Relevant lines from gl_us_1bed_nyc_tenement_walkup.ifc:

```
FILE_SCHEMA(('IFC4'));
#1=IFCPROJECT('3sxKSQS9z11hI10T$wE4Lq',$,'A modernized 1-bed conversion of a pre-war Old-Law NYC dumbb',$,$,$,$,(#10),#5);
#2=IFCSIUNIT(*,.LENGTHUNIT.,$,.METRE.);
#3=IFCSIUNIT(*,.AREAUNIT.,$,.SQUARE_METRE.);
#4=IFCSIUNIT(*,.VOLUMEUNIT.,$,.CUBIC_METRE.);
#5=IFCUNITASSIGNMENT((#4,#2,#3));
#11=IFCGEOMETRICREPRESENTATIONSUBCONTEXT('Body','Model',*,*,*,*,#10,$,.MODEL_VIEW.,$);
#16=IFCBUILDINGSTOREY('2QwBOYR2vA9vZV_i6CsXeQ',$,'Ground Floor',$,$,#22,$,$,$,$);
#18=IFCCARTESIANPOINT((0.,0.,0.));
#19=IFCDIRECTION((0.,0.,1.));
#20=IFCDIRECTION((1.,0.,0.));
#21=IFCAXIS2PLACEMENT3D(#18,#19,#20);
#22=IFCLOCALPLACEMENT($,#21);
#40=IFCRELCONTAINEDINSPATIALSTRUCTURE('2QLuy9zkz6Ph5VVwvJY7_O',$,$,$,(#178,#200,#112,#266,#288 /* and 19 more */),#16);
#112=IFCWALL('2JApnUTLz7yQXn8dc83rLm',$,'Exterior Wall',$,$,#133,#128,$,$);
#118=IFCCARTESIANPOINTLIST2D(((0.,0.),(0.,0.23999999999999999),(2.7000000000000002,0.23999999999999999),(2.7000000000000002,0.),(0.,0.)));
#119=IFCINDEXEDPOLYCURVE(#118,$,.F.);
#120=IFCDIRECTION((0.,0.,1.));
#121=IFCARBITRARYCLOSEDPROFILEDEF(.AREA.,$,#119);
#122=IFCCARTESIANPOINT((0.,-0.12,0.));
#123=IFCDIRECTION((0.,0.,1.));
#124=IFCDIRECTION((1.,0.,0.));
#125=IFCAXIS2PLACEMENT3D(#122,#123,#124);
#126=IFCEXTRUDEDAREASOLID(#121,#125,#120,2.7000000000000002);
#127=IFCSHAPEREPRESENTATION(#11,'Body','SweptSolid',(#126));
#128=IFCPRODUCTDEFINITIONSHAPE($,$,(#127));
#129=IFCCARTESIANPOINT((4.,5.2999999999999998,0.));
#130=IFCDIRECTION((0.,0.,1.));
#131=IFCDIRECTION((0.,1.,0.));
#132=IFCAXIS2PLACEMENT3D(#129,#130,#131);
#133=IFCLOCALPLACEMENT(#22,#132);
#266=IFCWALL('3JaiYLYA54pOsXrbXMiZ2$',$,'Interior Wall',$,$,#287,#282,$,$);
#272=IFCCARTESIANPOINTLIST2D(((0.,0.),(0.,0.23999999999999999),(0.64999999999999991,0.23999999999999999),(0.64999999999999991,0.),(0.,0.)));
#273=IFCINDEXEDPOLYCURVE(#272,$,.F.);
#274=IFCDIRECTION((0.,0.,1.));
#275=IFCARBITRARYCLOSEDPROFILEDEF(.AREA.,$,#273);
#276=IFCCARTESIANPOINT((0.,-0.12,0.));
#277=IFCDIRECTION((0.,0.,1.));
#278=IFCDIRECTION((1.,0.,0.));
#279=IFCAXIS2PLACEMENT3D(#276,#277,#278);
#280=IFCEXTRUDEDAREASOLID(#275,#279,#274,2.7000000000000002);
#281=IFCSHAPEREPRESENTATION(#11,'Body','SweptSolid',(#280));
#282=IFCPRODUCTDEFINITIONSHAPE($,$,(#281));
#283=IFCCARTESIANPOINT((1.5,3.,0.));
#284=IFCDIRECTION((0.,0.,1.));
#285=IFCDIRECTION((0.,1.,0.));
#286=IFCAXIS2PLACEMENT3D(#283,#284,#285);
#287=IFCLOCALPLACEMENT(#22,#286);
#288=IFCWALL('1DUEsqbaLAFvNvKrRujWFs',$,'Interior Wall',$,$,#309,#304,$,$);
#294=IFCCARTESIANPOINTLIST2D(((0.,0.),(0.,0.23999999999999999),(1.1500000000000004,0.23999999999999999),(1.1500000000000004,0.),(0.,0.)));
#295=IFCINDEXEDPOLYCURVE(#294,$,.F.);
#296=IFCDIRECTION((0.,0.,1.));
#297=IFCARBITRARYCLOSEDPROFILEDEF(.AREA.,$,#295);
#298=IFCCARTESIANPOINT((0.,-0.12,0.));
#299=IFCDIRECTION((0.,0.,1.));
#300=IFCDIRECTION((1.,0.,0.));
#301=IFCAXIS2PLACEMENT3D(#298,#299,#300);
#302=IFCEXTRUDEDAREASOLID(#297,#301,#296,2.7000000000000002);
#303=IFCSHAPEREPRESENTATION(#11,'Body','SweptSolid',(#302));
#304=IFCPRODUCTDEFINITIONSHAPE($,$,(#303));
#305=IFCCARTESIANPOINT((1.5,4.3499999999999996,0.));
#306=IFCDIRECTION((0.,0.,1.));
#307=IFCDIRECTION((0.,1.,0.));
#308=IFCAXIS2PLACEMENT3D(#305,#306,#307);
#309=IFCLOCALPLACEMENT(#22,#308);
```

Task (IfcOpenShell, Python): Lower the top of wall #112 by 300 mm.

```python
import ifcopenshell
import ifcopenshell.geom
import ifcopenshell.util.representation
import ifcopenshell.util.shape
import ifcopenshell.util.unit

model = ifcopenshell.open("gl_us_1bed_nyc_tenement_walkup.ifc")
unit_scale = ifcopenshell.util.unit.calculate_unit_scale(model)
settings = ifcopenshell.geom.settings()


def volume(element):
    """Net volume in cubic metres, openings subtracted."""
    shape = ifcopenshell.geom.create_shape(settings, element)
    return ifcopenshell.util.shape.get_volume(shape.geometry)


wall = model.by_guid("2JApnUTLz7yQXn8dc83rLm")
before = volume(wall)

body = ifcopenshell.util.representation.get_representation(wall, "Model", "Body")
solid = body.Items[0]
old_height = solid.Depth
solid.Depth -= 0.3 / unit_scale
after = volume(wall)

print(f"height {old_height:g} -> {solid.Depth:g}, volume {before:.3f} -> {after:.3f} m3")

model.write("gl_us_1bed_nyc_tenement_walkup_v2.ifc")
```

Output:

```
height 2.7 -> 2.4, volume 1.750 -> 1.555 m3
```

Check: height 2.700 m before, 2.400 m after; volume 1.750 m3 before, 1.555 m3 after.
